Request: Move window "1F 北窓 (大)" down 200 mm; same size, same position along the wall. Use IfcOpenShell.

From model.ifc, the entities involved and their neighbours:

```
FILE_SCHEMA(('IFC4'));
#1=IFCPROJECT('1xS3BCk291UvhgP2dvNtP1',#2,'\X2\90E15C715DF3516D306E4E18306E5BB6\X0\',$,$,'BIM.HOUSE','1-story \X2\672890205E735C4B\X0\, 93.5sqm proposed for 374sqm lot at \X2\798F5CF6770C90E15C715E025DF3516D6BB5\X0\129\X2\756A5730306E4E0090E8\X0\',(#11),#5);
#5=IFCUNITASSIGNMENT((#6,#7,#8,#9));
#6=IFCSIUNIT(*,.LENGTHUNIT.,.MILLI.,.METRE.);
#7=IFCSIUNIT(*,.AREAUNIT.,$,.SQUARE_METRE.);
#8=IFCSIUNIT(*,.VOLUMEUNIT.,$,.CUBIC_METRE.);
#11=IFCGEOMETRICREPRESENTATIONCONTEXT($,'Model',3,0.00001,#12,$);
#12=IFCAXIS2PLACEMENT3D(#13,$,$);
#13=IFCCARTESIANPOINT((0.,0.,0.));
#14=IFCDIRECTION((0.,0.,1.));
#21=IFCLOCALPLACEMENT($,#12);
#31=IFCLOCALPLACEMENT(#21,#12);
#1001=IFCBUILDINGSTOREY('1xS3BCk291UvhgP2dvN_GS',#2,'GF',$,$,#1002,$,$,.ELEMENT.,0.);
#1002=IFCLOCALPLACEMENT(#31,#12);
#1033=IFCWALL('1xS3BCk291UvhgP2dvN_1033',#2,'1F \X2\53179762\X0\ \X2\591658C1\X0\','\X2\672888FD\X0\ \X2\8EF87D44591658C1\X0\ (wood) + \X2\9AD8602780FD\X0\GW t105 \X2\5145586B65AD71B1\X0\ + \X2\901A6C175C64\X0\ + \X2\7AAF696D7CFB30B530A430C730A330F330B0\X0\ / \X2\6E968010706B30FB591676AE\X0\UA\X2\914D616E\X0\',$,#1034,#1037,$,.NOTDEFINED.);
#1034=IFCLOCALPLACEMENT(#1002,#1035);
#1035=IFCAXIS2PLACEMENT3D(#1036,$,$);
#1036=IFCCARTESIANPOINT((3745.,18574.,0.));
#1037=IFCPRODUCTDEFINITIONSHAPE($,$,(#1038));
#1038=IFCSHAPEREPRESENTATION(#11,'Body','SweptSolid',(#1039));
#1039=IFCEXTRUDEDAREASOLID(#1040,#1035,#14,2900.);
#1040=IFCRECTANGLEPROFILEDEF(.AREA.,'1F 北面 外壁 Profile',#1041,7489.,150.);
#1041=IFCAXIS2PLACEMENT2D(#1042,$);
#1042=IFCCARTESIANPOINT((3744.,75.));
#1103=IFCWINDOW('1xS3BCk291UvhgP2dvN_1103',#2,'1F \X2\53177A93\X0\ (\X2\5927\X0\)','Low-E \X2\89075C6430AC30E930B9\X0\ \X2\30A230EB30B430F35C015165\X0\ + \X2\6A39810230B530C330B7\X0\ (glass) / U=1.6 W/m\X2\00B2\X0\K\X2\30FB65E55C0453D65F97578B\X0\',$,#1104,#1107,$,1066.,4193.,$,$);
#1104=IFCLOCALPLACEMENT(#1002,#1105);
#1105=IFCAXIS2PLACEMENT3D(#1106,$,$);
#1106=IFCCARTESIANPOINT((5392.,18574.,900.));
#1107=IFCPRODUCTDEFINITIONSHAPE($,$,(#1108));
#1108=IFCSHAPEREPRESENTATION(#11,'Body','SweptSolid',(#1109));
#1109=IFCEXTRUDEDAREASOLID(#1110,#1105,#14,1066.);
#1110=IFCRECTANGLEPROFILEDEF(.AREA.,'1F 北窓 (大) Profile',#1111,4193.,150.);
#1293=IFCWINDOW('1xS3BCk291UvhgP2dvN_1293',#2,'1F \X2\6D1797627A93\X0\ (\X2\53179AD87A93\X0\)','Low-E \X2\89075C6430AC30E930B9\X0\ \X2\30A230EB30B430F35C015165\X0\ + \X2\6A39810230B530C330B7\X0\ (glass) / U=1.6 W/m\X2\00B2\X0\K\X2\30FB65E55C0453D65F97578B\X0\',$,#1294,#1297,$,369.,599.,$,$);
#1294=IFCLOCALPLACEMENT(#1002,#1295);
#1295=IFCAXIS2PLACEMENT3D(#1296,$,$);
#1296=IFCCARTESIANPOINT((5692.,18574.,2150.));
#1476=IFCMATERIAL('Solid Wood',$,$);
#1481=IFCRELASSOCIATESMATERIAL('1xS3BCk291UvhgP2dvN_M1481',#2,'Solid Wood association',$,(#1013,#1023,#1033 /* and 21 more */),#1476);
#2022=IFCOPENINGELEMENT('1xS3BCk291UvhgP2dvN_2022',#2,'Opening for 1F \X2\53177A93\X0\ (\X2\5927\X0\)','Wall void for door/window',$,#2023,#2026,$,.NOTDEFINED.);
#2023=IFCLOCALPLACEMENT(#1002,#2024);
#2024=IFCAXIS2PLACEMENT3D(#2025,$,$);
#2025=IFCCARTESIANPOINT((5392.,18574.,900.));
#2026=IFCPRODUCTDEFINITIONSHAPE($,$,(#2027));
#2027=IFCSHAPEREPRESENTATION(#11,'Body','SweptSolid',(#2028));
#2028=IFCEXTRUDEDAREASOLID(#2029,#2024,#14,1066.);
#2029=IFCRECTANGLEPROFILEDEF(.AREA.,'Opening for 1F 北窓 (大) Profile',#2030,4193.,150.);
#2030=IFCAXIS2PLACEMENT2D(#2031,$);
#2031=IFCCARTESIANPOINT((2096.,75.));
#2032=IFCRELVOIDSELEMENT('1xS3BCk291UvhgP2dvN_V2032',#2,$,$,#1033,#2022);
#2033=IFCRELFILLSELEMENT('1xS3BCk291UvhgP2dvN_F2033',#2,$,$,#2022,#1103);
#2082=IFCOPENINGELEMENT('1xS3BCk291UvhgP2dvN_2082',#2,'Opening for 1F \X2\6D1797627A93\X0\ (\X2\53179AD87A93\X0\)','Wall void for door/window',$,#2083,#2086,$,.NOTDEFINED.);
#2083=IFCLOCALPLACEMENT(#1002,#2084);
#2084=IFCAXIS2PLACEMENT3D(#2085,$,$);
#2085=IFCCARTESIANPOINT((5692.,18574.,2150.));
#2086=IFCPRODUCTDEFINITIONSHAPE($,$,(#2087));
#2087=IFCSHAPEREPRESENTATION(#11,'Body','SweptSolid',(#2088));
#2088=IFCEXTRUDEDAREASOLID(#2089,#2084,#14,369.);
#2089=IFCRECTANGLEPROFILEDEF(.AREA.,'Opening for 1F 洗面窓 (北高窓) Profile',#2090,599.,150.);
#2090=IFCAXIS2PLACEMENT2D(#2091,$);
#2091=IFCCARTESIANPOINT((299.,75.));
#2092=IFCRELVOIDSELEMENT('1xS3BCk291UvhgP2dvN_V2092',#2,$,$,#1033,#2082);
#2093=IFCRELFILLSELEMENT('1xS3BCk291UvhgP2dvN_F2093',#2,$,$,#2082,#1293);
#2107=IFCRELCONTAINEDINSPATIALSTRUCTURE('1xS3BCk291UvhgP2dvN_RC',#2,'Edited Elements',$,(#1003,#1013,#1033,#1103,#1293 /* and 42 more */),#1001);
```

```python
import numpy as np
import ifcopenshell
import ifcopenshell.api.geometry
import ifcopenshell.util.placement
import ifcopenshell.util.unit

model = ifcopenshell.open("model.ifc")
unit_scale = ifcopenshell.util.unit.calculate_unit_scale(model)

window = model.by_id(1103)
opening = window.FillsVoids[0].RelatingOpeningElement
dz = -0.2 / unit_scale

shift = np.array([0.0, 0.0, dz])
# The window is not placed relative to its opening, so move both.
for product in (opening, window):
    matrix = ifcopenshell.util.placement.get_local_placement(product.ObjectPlacement)
    matrix[:3, 3] += shift
    ifcopenshell.api.geometry.edit_object_placement(model, product=product, matrix=matrix, is_si=False)

print(f"moved by {dz * unit_scale:+.3f} m")

model.write("model_edited.ifc")
```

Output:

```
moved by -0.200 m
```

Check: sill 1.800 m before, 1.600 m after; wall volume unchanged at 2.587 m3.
